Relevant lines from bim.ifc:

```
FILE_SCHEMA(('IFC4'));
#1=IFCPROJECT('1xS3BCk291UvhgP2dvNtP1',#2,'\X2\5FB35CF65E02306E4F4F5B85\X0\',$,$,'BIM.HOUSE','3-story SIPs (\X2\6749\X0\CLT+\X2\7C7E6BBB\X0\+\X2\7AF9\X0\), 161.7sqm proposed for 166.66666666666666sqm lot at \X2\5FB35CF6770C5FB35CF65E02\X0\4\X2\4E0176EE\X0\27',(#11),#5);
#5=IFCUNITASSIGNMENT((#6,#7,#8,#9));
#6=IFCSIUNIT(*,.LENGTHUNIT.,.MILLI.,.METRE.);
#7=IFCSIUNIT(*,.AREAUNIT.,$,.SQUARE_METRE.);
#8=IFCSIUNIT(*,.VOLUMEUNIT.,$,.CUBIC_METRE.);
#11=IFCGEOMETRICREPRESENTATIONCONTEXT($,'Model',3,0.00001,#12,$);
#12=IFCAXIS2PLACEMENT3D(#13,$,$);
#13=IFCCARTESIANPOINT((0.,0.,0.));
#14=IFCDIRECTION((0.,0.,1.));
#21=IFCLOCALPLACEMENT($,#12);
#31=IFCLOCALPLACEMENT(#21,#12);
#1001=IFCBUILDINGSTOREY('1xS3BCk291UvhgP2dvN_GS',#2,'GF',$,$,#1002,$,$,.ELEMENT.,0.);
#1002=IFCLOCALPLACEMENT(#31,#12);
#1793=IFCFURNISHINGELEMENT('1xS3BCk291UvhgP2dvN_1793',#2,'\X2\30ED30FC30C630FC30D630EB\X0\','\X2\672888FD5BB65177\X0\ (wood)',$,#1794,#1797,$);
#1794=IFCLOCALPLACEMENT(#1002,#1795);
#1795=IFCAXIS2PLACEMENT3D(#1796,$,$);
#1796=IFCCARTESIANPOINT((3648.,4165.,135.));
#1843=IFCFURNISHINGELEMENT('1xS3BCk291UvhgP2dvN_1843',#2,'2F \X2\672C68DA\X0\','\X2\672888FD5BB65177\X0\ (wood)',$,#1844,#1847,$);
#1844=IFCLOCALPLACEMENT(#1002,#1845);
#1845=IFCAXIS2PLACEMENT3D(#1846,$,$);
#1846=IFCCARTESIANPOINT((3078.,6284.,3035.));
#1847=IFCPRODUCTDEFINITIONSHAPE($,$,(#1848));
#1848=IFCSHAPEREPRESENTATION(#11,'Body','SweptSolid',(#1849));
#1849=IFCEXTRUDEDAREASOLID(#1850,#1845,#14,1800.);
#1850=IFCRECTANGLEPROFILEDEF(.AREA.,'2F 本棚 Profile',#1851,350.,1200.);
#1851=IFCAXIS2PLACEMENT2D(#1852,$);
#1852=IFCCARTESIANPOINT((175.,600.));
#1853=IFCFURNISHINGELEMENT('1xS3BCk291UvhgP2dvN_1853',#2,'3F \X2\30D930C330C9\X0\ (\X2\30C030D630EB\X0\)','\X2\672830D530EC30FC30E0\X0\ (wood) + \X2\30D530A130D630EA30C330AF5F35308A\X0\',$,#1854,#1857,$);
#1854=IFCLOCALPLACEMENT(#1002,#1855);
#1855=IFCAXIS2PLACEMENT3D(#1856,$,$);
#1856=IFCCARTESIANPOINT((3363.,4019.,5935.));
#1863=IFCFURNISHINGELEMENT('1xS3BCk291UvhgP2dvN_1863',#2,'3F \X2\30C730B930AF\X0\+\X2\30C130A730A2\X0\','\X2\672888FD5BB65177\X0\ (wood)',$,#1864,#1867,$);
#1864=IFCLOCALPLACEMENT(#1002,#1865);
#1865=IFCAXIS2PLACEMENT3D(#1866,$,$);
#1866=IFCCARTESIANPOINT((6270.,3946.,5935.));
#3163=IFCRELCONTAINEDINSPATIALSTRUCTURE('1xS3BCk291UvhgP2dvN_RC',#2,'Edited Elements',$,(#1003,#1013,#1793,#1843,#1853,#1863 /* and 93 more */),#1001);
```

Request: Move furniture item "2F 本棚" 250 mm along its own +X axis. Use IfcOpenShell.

```python
import ifcopenshell
import ifcopenshell.api.geometry
import ifcopenshell.util.placement

model = ifcopenshell.open("bim.ifc")

item = model.by_guid("1xS3BCk291UvhgP2dvN_1843")
matrix = ifcopenshell.util.placement.get_local_placement(item.ObjectPlacement)
matrix[:3, 3] += matrix[:3, 0] * 250.0
ifcopenshell.api.geometry.edit_object_placement(model, product=item, matrix=matrix, is_si=False)

print(ifcopenshell.util.placement.get_local_placement(item.ObjectPlacement).round(3) + 0.0)

model.write("bim_v2.ifc")
```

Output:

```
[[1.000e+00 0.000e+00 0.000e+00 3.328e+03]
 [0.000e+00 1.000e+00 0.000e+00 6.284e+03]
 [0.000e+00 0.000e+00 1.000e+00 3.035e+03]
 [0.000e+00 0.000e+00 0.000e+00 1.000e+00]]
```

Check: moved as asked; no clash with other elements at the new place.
